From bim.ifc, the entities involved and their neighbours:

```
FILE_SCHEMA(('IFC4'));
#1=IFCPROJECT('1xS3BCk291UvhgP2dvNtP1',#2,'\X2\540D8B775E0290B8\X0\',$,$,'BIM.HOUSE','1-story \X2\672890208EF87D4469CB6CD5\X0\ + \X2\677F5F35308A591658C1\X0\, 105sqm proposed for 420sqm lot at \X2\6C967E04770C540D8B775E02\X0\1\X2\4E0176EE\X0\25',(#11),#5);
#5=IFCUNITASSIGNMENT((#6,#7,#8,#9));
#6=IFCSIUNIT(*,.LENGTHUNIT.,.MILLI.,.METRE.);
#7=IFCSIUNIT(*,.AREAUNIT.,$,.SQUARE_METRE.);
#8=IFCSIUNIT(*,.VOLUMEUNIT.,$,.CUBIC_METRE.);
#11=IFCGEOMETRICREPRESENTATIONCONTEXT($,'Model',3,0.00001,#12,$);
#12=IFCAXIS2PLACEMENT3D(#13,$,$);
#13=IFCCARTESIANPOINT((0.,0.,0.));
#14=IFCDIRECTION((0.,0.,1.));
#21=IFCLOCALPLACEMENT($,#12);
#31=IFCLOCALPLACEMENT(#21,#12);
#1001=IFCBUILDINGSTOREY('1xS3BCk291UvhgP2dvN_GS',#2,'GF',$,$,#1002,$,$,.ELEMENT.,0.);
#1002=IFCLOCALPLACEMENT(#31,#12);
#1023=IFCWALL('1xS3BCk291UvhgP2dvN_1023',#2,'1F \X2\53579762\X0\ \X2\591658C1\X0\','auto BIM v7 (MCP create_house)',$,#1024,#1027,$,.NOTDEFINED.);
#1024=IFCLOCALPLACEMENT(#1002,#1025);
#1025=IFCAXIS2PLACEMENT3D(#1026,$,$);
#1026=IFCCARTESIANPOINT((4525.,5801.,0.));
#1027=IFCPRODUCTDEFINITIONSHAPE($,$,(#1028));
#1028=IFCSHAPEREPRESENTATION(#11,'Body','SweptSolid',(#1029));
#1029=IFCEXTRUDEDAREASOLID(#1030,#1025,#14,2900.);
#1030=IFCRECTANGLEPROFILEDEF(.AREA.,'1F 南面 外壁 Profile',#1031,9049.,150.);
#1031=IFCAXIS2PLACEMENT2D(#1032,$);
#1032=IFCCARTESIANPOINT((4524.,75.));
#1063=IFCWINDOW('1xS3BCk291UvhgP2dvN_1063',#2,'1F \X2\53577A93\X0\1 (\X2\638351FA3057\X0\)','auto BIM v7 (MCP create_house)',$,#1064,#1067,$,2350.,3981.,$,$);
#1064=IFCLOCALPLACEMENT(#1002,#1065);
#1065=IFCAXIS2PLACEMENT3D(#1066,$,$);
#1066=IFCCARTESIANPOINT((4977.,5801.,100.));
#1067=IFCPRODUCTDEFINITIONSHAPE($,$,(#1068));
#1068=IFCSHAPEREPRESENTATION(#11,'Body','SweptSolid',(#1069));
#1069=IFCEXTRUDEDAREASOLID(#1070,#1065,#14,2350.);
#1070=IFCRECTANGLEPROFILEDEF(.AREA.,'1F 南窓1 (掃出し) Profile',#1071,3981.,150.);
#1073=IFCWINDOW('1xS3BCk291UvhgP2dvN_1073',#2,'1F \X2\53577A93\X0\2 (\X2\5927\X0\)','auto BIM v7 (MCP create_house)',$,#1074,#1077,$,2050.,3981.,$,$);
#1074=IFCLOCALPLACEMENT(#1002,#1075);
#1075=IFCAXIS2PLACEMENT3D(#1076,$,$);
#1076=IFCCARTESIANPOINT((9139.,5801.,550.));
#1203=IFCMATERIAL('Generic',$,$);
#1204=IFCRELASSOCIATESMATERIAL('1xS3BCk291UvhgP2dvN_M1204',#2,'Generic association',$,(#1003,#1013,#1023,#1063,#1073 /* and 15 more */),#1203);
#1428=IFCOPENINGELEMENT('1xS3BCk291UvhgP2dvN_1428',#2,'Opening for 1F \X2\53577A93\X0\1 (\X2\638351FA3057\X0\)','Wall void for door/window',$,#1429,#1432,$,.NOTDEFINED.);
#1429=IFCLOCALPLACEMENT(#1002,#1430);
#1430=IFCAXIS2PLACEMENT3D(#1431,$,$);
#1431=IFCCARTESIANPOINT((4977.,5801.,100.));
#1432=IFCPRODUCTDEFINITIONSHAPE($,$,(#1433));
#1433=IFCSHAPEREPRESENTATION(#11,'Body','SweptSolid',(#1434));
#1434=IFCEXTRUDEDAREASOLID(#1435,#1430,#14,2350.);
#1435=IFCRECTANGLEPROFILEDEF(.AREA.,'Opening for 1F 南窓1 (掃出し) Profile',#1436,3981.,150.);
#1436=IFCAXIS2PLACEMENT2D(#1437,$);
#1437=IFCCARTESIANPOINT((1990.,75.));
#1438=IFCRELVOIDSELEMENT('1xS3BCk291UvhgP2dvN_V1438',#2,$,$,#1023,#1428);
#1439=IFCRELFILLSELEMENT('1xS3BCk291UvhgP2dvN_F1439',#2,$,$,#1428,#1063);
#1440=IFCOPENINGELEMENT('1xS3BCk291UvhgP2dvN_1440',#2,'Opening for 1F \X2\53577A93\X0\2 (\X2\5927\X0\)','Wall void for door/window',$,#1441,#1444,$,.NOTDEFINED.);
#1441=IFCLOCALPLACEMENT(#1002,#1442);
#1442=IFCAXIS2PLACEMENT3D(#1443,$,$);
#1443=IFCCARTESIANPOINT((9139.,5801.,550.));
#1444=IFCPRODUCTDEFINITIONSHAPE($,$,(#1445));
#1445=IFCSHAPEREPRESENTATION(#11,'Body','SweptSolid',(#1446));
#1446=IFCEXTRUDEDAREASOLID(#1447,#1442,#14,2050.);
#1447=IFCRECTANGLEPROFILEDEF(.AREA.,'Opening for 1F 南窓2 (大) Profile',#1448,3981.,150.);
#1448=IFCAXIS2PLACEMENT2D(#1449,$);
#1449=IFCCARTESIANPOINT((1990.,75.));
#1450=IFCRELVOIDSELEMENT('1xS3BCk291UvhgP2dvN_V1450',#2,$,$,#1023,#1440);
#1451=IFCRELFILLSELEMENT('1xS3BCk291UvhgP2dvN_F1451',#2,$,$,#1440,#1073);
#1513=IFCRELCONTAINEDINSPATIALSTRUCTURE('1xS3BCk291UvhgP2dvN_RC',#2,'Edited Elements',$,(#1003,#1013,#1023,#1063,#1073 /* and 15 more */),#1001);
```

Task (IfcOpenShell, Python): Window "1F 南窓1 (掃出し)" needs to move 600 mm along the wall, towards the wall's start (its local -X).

```python
import ifcopenshell
import ifcopenshell.api.geometry
import ifcopenshell.util.placement
import ifcopenshell.util.unit

model = ifcopenshell.open("bim.ifc")
unit_scale = ifcopenshell.util.unit.calculate_unit_scale(model)

window = model.by_id(1063)
opening = window.FillsVoids[0].RelatingOpeningElement
wall = opening.VoidsElements[0].RelatingBuildingElement

wall_matrix = ifcopenshell.util.placement.get_local_placement(wall.ObjectPlacement)
shift = wall_matrix[:3, 0] * -0.6 / unit_scale
before = ifcopenshell.util.placement.get_local_placement(window.ObjectPlacement)[:3, 3].copy()

# The window is not placed relative to its opening, so move both.
for product in (opening, window):
    matrix = ifcopenshell.util.placement.get_local_placement(product.ObjectPlacement)
    matrix[:3, 3] += shift
    ifcopenshell.api.geometry.edit_object_placement(model, product=product, matrix=matrix, is_si=False)

after = ifcopenshell.util.placement.get_local_placement(window.ObjectPlacement)[:3, 3]
print("window moved by", (after - before).round(3) + 0.0)

model.write("bim_updated.ifc")
```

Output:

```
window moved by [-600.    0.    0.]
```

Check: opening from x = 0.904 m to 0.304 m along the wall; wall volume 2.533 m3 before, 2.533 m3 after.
